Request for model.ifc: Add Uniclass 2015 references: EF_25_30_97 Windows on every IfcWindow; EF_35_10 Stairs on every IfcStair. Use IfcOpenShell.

First a look at what the model holds.

```python
import ifcopenshell

model = ifcopenshell.open("model.ifc")
print(model.schema)
print("classifications:", [c.Name for c in model.by_type("IfcClassification")])
for ifc_class in ("IfcDoor", "IfcRoof", "IfcStair", "IfcWall", "IfcWindow"):
    print(ifc_class, len(model.by_type(ifc_class)))
```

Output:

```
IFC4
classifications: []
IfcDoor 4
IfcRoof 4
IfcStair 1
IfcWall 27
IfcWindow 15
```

```python
import ifcopenshell
import ifcopenshell.api.classification

model = ifcopenshell.open("model.ifc")

system = ifcopenshell.api.classification.add_classification(model, classification="Uniclass 2015")

codes = {
    "IfcWindow": ("EF_25_30_97", "Windows"),
    "IfcStair": ("EF_35_10", "Stairs"),
}
for ifc_class, (code, name) in codes.items():
    products = model.by_type(ifc_class)
    ifcopenshell.api.classification.add_reference(
        model, products=products, classification=system, identification=code, name=name
    )
    print(code, len(products))

model.write("model_updated.ifc")
```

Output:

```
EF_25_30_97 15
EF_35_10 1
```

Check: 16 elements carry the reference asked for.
